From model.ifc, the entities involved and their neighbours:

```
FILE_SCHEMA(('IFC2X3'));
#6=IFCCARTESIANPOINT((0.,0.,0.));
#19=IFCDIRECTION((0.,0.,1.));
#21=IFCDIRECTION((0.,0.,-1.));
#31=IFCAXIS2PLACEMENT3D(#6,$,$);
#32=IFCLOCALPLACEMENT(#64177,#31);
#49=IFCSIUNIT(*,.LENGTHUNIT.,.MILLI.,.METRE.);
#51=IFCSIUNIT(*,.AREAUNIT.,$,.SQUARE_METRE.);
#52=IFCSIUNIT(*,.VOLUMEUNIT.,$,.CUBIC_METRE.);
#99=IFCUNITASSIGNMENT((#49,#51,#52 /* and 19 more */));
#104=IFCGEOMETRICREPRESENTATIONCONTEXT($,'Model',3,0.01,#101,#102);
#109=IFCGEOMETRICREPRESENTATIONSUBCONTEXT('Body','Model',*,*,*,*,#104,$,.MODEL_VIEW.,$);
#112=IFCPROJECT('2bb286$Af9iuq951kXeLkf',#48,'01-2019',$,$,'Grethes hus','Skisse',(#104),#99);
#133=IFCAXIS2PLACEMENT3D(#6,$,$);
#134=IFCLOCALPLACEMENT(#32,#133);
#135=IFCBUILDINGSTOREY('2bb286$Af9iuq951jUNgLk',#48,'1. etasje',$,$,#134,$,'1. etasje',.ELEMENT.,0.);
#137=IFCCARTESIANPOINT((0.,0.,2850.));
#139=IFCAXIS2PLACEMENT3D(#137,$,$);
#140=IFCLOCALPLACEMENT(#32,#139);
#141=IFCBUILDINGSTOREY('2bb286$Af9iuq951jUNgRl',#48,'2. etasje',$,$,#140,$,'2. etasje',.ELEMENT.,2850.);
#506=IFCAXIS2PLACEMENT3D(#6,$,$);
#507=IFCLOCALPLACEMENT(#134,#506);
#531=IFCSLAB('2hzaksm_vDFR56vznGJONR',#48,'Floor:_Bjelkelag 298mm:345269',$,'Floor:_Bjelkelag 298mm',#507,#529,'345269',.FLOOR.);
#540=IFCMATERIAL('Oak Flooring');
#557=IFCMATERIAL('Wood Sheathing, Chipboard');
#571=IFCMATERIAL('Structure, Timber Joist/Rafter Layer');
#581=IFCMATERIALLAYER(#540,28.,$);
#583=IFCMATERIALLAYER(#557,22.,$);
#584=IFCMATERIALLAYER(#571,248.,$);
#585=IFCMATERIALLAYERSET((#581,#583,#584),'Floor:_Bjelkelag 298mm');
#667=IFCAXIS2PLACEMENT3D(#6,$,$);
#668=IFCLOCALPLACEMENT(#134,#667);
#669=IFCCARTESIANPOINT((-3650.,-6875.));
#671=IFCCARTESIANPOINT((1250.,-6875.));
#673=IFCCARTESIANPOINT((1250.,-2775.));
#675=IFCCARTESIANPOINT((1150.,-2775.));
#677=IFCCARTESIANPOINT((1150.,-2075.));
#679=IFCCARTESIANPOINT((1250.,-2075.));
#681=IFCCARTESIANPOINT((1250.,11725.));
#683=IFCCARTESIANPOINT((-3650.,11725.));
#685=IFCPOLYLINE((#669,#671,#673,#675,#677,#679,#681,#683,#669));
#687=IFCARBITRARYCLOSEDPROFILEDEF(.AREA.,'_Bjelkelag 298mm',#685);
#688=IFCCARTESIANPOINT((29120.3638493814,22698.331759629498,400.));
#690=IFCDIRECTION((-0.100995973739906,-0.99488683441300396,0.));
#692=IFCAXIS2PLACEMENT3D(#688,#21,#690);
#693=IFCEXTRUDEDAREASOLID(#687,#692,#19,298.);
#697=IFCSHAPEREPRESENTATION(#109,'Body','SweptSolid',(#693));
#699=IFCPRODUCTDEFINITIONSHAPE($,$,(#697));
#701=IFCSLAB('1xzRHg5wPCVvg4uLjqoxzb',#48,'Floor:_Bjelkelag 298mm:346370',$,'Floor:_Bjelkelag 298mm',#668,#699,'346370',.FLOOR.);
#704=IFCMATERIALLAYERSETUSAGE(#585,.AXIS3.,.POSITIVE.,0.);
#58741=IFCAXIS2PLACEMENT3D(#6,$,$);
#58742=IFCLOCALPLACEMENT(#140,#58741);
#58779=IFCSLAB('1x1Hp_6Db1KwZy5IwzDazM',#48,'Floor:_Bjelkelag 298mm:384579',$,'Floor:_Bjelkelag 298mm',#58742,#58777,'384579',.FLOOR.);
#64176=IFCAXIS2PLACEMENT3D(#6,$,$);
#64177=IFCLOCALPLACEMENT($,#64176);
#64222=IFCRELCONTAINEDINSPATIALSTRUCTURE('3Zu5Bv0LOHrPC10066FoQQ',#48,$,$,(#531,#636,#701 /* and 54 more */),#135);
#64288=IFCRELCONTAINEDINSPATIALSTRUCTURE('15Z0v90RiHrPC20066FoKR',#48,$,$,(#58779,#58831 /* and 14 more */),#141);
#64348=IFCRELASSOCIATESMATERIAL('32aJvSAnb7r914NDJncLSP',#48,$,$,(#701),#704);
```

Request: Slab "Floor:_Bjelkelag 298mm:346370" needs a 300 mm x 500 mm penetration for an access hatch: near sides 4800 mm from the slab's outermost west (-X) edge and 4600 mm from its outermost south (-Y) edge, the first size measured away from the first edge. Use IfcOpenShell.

```python
import numpy as np
import ifcopenshell
import ifcopenshell.api.feature
import ifcopenshell.api.geometry
import ifcopenshell.api.root
import ifcopenshell.geom
import ifcopenshell.util.placement
import ifcopenshell.util.representation
import ifcopenshell.util.shape
import ifcopenshell.util.unit

model = ifcopenshell.open("model.ifc")
unit_scale = ifcopenshell.util.unit.calculate_unit_scale(model)
settings = ifcopenshell.geom.settings()


def volume(element):
    """Net volume in cubic metres, openings subtracted."""
    shape = ifcopenshell.geom.create_shape(settings, element)
    return ifcopenshell.util.shape.get_volume(shape.geometry)


slab = model.by_id(701)
before = volume(slab)

# Extent in the slab's own axes, in metres. The edges named are its -X and -Y sides.
slab_shape = ifcopenshell.geom.create_shape(settings, slab)
vertices = ifcopenshell.util.shape.get_vertices(slab_shape.geometry)
x_min, y_min, bottom = vertices.min(axis=0)
top = vertices[:, 2].max()

opening = ifcopenshell.api.root.create_entity(model, ifc_class="IfcOpeningElement", name="Access hatch opening")
context = ifcopenshell.util.representation.get_context(model, "Model", "Body", "MODEL_VIEW")
width, depth = 0.3, 0.5
outline = [(0.0, 0.0), (width, 0.0), (width, depth), (0.0, depth), (0.0, 0.0)]
# Overshoot both faces by 50 mm so the cut is clean.
shape = ifcopenshell.api.geometry.add_slab_representation(
    model, context=context, depth=top - bottom + 0.1, polyline=outline
)
ifcopenshell.api.geometry.assign_representation(model, product=opening, representation=shape)

matrix = ifcopenshell.util.placement.get_local_placement(slab.ObjectPlacement)
matrix[:, 3] = matrix @ np.append(np.array([x_min + 4.8, y_min + 4.6, bottom - 0.05]) / unit_scale, 1.0)
ifcopenshell.api.geometry.edit_object_placement(model, product=opening, matrix=matrix, is_si=False)
ifcopenshell.api.feature.add_feature(model, feature=opening, element=slab)

after = volume(slab)

print(f"slab volume {before:.3f} -> {after:.3f} m3")

model.write("model_edited.ifc")
```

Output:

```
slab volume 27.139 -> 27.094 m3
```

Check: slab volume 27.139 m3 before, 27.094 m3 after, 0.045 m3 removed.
